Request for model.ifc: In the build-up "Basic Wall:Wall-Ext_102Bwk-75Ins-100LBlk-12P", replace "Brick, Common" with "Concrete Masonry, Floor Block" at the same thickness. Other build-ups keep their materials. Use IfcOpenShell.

First a look at what the model holds.

```python
import ifcopenshell
import ifcopenshell.util.element

model = ifcopenshell.open("model.ifc")
print(model.schema)
for layer_set in model.by_type("IfcMaterialLayerSet"):
    if layer_set.LayerSetName == "Basic Wall:Wall-Ext_102Bwk-75Ins-100LBlk-12P":
        for layer in layer_set.MaterialLayers:
            print(layer.id(), layer.Material and layer.Material.Name, layer.LayerThickness, sep=" | ")
        print(len(ifcopenshell.util.element.get_elements_by_material(model, layer_set)), "elements and types use it")
print(sorted(m.Name for m in model.by_type("IfcMaterial") if m.Name)[:60])
```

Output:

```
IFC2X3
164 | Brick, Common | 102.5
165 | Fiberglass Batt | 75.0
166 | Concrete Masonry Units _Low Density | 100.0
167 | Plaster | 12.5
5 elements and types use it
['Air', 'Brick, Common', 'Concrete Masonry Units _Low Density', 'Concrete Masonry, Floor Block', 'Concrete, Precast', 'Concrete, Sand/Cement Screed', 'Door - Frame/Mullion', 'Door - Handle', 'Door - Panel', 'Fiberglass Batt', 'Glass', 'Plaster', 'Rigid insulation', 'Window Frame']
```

```python
import ifcopenshell
import ifcopenshell.api.material

model = ifcopenshell.open("model.ifc")

layer_set = next(s for s in model.by_type("IfcMaterialLayerSet") if s.LayerSetName == "Basic Wall:Wall-Ext_102Bwk-75Ins-100LBlk-12P")
layer = next(l for l in layer_set.MaterialLayers if l.Material and l.Material.Name == "Brick, Common")
material = next(m for m in model.by_type("IfcMaterial") if m.Name == "Concrete Masonry, Floor Block")

# Point this one layer at the other material; renaming the old one would change it everywhere.
ifcopenshell.api.material.edit_layer(model, layer=layer, attributes={}, material=material)

print([l.Material.Name if l.Material else None for l in layer_set.MaterialLayers])

model.write("model-out.ifc")
```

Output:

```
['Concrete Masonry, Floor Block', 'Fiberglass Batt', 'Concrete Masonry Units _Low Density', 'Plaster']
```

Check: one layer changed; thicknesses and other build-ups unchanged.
